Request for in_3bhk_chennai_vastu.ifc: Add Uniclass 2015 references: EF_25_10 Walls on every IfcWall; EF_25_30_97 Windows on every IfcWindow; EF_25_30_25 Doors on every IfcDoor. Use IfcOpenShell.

First a look at what the model holds.

```python
import ifcopenshell

model = ifcopenshell.open("in_3bhk_chennai_vastu.ifc")
print(model.schema)
print("classifications:", [c.Name for c in model.by_type("IfcClassification")])
for ifc_class in ("IfcDoor", "IfcRoof", "IfcStair", "IfcWall", "IfcWindow"):
    print(ifc_class, len(model.by_type(ifc_class)))
```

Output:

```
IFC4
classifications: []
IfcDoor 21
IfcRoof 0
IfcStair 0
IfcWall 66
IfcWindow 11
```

```python
import ifcopenshell
import ifcopenshell.api.classification

model = ifcopenshell.open("in_3bhk_chennai_vastu.ifc")

system = ifcopenshell.api.classification.add_classification(model, classification="Uniclass 2015")

codes = {
    "IfcWall": ("EF_25_10", "Walls"),
    "IfcWindow": ("EF_25_30_97", "Windows"),
    "IfcDoor": ("EF_25_30_25", "Doors"),
}
for ifc_class, (code, name) in codes.items():
    products = model.by_type(ifc_class)
    ifcopenshell.api.classification.add_reference(
        model, products=products, classification=system, identification=code, name=name
    )
    print(code, len(products))

model.write("in_3bhk_chennai_vastu_v2.ifc")
```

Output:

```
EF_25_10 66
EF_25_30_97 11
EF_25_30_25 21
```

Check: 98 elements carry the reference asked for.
